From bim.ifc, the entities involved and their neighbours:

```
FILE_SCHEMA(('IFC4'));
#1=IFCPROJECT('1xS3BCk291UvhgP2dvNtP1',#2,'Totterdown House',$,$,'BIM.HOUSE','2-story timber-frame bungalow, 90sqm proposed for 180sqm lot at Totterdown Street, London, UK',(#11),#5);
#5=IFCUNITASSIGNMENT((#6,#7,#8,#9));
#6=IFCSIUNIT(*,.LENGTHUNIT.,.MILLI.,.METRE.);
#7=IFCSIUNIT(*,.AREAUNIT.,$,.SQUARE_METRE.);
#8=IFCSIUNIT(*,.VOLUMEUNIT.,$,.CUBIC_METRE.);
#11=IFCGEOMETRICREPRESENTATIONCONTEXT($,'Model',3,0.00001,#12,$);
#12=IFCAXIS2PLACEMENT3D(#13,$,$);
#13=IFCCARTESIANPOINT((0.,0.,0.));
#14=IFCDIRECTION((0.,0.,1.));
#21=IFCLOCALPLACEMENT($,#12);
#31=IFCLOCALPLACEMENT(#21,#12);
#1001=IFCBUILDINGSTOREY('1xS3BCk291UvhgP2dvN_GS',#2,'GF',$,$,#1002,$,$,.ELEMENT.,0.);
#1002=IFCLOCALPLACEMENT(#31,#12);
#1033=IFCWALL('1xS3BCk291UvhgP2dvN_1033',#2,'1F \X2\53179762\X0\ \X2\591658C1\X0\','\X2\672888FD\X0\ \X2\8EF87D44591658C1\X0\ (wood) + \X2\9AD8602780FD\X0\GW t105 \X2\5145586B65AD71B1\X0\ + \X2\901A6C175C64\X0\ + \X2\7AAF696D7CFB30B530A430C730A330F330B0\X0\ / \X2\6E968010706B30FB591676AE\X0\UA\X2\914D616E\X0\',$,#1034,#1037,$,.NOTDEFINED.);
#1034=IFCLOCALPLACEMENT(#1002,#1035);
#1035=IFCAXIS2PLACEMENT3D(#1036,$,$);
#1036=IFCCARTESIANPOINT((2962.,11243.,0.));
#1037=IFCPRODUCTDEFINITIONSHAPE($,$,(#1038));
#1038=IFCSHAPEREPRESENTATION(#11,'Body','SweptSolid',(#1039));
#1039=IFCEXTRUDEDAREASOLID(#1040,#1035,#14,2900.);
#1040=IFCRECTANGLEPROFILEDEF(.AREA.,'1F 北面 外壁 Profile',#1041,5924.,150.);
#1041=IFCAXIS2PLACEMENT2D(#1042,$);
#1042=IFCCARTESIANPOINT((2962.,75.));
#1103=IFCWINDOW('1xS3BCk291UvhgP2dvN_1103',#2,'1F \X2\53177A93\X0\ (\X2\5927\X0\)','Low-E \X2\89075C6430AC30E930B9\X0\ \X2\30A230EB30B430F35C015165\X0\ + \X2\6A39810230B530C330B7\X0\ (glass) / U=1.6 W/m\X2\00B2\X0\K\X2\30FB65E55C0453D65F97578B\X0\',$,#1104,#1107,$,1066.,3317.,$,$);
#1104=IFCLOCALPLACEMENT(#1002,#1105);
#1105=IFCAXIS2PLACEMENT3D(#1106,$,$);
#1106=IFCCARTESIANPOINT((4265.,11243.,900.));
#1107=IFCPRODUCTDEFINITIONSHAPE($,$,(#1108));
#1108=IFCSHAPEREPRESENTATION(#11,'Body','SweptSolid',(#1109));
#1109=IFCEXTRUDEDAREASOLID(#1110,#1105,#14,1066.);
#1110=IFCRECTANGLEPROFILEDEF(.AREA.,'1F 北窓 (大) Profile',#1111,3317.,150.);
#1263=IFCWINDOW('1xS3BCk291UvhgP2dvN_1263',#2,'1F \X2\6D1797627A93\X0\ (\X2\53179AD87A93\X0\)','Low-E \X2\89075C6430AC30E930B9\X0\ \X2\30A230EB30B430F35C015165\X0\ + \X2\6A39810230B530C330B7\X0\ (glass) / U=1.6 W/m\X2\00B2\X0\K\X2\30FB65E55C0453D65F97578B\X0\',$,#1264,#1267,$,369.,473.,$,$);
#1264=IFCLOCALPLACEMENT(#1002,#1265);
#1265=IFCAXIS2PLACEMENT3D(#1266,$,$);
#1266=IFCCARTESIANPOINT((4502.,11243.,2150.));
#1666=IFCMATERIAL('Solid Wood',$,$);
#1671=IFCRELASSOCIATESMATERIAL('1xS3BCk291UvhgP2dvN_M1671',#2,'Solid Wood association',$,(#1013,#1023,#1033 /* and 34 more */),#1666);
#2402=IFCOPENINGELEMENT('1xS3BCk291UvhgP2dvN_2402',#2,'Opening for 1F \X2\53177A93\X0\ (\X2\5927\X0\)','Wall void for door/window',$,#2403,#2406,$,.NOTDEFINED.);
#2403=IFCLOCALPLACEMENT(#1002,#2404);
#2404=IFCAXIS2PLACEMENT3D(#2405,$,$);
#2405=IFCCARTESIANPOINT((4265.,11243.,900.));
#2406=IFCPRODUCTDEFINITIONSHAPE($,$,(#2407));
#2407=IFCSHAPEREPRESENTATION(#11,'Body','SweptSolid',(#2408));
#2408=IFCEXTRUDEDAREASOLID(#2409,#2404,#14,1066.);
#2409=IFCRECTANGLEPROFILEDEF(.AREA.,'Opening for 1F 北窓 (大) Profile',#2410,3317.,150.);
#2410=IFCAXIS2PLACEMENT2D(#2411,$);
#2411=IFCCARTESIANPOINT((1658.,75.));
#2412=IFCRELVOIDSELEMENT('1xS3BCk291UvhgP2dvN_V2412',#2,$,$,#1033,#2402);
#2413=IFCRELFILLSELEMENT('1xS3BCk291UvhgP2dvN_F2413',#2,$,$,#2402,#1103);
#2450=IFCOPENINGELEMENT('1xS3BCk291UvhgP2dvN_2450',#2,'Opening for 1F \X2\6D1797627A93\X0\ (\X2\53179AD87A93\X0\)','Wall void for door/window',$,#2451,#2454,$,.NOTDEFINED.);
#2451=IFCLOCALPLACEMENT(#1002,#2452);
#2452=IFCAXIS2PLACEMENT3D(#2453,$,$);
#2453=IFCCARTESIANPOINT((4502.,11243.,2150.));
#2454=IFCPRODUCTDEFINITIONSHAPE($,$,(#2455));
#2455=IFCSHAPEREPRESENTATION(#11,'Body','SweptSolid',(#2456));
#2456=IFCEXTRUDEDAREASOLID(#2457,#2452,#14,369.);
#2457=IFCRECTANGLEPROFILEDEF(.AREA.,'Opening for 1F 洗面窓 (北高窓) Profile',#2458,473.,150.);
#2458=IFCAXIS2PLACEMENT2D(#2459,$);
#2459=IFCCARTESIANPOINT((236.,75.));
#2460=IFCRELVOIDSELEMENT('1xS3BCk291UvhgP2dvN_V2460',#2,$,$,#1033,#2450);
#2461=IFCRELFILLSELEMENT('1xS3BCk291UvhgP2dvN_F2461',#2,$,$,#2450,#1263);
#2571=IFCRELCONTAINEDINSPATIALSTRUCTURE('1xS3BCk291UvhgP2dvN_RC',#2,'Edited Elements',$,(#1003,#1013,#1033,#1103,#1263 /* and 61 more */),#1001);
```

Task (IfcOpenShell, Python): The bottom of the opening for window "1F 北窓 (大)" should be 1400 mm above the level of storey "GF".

```python
import numpy as np
import ifcopenshell
import ifcopenshell.api.geometry
import ifcopenshell.geom
import ifcopenshell.util.element
import ifcopenshell.util.placement
import ifcopenshell.util.shape
import ifcopenshell.util.unit

model = ifcopenshell.open("bim.ifc")
unit_scale = ifcopenshell.util.unit.calculate_unit_scale(model)

window = model.by_id(1103)
opening = window.FillsVoids[0].RelatingOpeningElement
storey = ifcopenshell.util.element.get_container(window, ifc_class="IfcBuildingStorey")
level = ifcopenshell.util.placement.get_local_placement(storey.ObjectPlacement)[2, 3]

# The opening's origin need not be at the sill, so measure its lowest point.
shape = ifcopenshell.geom.create_shape(ifcopenshell.geom.settings(), opening)
bottom = ifcopenshell.util.shape.get_shape_bottom_elevation(shape, shape.geometry) / unit_scale
dz = level + 1400.0 - bottom

shift = np.array([0.0, 0.0, dz])
# The window is not placed relative to its opening, so move both.
for product in (opening, window):
    matrix = ifcopenshell.util.placement.get_local_placement(product.ObjectPlacement)
    matrix[:3, 3] += shift
    ifcopenshell.api.geometry.edit_object_placement(model, product=product, matrix=matrix, is_si=False)

print(f"moved by {dz * unit_scale:+.3f} m")

model.write("bim_edited.ifc")
```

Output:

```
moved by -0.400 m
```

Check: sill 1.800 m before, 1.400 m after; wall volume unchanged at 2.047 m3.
